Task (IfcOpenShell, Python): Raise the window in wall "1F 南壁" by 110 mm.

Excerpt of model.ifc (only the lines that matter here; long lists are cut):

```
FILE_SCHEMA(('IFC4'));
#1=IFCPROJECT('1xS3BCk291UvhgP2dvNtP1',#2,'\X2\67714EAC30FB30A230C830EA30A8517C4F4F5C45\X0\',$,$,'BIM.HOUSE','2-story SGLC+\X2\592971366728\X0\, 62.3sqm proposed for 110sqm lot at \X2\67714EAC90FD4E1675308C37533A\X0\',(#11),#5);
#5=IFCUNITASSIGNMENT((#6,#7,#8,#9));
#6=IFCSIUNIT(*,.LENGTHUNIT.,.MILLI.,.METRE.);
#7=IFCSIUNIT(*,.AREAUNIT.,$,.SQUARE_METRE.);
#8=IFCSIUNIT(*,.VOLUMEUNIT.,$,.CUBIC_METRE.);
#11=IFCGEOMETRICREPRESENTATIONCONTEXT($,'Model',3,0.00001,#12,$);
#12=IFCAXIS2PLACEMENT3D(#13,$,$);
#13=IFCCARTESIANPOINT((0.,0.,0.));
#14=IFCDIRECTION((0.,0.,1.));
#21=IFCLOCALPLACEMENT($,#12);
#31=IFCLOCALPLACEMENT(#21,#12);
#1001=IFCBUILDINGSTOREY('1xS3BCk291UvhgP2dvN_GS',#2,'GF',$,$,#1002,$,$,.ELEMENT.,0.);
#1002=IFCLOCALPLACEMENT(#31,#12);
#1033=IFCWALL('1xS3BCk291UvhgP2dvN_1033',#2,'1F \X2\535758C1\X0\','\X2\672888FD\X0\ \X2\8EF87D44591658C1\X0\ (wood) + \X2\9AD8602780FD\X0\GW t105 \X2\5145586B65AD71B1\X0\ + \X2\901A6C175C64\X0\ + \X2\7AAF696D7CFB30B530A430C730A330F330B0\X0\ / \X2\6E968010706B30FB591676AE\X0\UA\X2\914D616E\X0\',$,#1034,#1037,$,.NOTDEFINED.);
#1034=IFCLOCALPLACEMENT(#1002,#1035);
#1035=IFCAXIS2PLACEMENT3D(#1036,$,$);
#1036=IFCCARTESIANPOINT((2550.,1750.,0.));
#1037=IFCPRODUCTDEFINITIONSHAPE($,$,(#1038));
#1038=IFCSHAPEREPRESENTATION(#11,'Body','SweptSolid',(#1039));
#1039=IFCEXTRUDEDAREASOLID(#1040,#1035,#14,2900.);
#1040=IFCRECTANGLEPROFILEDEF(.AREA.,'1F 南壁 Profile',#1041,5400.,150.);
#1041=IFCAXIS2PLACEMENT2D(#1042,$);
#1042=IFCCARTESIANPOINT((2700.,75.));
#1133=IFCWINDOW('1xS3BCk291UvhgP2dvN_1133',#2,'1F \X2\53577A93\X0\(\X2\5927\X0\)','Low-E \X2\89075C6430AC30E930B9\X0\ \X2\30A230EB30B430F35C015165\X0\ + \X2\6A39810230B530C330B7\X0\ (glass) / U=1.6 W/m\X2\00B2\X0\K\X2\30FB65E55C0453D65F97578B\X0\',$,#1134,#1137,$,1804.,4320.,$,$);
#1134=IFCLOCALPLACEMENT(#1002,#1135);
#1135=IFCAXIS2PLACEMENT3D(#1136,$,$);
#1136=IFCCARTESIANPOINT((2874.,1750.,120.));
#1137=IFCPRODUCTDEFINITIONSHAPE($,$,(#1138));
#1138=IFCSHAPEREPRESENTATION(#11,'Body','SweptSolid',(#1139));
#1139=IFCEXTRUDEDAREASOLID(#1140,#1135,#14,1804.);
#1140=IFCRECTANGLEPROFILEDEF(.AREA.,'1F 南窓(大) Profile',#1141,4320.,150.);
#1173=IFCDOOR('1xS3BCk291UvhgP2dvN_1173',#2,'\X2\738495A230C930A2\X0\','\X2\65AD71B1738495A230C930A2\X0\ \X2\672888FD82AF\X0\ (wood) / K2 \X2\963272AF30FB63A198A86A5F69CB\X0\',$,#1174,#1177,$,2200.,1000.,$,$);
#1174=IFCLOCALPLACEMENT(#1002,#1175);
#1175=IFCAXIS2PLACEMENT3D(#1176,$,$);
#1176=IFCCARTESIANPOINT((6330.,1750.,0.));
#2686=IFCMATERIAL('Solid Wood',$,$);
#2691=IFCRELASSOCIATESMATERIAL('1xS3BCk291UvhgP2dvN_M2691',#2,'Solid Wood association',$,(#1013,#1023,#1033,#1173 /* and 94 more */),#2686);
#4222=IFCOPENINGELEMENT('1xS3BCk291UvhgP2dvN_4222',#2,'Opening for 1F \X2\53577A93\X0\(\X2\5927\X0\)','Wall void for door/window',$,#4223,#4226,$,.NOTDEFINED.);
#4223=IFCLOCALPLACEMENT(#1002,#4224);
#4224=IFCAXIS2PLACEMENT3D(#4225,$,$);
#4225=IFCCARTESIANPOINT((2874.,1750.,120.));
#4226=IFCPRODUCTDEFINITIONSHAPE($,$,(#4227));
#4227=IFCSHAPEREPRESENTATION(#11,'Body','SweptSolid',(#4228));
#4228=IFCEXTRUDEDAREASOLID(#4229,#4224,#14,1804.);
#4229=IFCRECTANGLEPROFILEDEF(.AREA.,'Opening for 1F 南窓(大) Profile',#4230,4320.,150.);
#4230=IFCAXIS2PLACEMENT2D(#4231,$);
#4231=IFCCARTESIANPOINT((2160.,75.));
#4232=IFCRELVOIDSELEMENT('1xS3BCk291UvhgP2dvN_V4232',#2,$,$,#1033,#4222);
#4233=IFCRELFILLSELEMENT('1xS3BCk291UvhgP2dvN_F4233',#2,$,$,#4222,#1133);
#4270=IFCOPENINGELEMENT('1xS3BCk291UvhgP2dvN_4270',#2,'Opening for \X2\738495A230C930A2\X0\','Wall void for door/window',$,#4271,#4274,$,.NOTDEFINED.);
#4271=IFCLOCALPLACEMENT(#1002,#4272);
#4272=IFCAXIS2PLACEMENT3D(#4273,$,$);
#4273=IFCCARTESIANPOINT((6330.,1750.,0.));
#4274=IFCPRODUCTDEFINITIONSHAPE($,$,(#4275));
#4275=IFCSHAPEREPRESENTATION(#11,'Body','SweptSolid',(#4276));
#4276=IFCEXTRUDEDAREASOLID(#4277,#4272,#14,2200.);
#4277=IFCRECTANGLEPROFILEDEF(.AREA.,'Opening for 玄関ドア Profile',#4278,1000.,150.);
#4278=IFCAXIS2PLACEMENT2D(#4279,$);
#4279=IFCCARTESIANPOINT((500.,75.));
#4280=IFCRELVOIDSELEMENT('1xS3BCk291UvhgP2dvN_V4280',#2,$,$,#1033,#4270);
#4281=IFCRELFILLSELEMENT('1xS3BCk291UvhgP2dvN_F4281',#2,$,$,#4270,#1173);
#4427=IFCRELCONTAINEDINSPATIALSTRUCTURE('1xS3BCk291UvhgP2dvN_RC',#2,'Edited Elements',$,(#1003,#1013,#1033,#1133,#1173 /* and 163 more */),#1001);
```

```python
import numpy as np
import ifcopenshell
import ifcopenshell.api.geometry
import ifcopenshell.util.placement
import ifcopenshell.util.unit

model = ifcopenshell.open("model.ifc")
unit_scale = ifcopenshell.util.unit.calculate_unit_scale(model)

window = model.by_id(1133)
opening = window.FillsVoids[0].RelatingOpeningElement
dz = 110.0

shift = np.array([0.0, 0.0, dz])
# The window is not placed relative to its opening, so move both.
for product in (opening, window):
    matrix = ifcopenshell.util.placement.get_local_placement(product.ObjectPlacement)
    matrix[:3, 3] += shift
    ifcopenshell.api.geometry.edit_object_placement(model, product=product, matrix=matrix, is_si=False)

print(f"moved by {dz * unit_scale:+.3f} m")

model.write("model_v2.ifc")
```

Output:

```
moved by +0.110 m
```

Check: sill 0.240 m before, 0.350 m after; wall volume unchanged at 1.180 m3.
